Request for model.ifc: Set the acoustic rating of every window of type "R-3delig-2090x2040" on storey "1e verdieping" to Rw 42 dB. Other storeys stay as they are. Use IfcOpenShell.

First a look at what the model holds.

```python
import ifcopenshell
import ifcopenshell.util.element

model = ifcopenshell.open("model.ifc")
print(model.schema)
storey = next(s for s in model.by_type("IfcBuildingStorey") if s.Name == "1e verdieping")
windows = [e for e in ifcopenshell.util.element.get_decomposition(storey) if e.is_a("IfcWindow")]
seen = {}
for e in windows:
    element_type = ifcopenshell.util.element.get_type(e)
    key = (element_type.Name if element_type != e and element_type else None, ifcopenshell.util.element.get_pset(e, "Pset_WindowCommon", "AcousticRating"))
    seen[key] = seen.get(key, 0) + 1
for (name, value), count in sorted(seen.items(), key=str):
    print(count, "x", name, "|", value)
```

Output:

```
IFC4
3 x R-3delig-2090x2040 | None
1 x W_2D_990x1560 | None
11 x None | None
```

```python
import ifcopenshell
import ifcopenshell.api.pset
import ifcopenshell.util.element

model = ifcopenshell.open("model.ifc")

storey = next(s for s in model.by_type("IfcBuildingStorey") if s.Name == "1e verdieping")
windows = [e for e in ifcopenshell.util.element.get_decomposition(storey) if e.is_a("IfcWindow")]

count = 0
for e in windows:
    element_type = ifcopenshell.util.element.get_type(e)
    if element_type in (None, e) or element_type.Name != "R-3delig-2090x2040":
        continue
    # add_pset returns the element's existing set when there is one.
    pset = ifcopenshell.api.pset.add_pset(model, product=e, name="Pset_WindowCommon")
    ifcopenshell.api.pset.edit_pset(model, pset=pset, properties={"AcousticRating": "Rw 42 dB"})
    count += 1

print(count, "windows updated")

model.write("model_updated.ifc")
```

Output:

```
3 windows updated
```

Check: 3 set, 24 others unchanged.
